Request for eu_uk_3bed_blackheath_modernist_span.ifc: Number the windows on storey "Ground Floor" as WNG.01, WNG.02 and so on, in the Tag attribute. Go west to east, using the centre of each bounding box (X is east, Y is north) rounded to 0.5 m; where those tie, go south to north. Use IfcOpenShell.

First a look at what the model holds.

```python
import ifcopenshell
import ifcopenshell.util.element
import ifcopenshell.util.placement

model = ifcopenshell.open("eu_uk_3bed_blackheath_modernist_span.ifc")
print(model.schema)
storey = next(s for s in model.by_type("IfcBuildingStorey") if s.Name == "Ground Floor")
windows = [e for e in ifcopenshell.util.element.get_decomposition(storey) if e.is_a("IfcWindow")]
for e in sorted(windows, key=lambda e: e.id()):
    origin = ifcopenshell.util.placement.get_local_placement(e.ObjectPlacement)[:3, 3]
    print(e.id(), e.Tag, e.Name, origin.round(2) + 0.0, sep=" | ")
```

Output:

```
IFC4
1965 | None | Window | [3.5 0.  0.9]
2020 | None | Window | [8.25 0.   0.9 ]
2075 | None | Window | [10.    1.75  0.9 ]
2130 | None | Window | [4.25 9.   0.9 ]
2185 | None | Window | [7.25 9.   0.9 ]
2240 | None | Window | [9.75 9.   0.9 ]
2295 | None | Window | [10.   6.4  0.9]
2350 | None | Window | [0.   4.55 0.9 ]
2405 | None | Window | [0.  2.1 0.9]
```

```python
import ifcopenshell
import ifcopenshell.geom
import ifcopenshell.util.element
import ifcopenshell.util.shape

model = ifcopenshell.open("eu_uk_3bed_blackheath_modernist_span.ifc")
settings = ifcopenshell.geom.settings()
settings.set("use-world-coords", True)


def centre(element):
    shape = ifcopenshell.geom.create_shape(settings, element)
    return ifcopenshell.util.shape.get_bbox_centroid(shape.geometry)


storey = next(s for s in model.by_type("IfcBuildingStorey") if s.Name == "Ground Floor")
windows = [e for e in ifcopenshell.util.element.get_decomposition(storey) if e.is_a("IfcWindow")]

# Insertion points can sit at a corner or the storey origin, so sort by the geometry (in metres).
centres = {e: centre(e) for e in windows}
windows.sort(key=lambda e: (round(centres[e][0] / 0.5), centres[e][1]))

for i, e in enumerate(windows, start=1):
    number = f"WNG.{i:02d}"
    e.Tag = number
    print(e.id(), number)

model.write("eu_uk_3bed_blackheath_modernist_span-out.ifc")
```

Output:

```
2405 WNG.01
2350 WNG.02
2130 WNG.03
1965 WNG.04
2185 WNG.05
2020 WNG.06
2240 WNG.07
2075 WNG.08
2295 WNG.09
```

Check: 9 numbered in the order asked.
